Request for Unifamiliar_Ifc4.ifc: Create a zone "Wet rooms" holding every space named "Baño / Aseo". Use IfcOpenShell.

First a look at what the model holds.

```python
import ifcopenshell

model = ifcopenshell.open("Unifamiliar_Ifc4.ifc")
print(model.schema)
seen = {}
for space in model.by_type("IfcSpace"):
    seen[space.LongName] = seen.get(space.LongName, 0) + 1
for name, count in sorted(seen.items(), key=str):
    print(count, "x", name)
print("zones:", [z.Name for z in model.by_type("IfcZone")][:20])
```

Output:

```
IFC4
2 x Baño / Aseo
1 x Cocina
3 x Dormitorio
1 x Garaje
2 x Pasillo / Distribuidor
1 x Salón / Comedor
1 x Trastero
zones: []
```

```python
import ifcopenshell
import ifcopenshell.api.group
import ifcopenshell.api.root

model = ifcopenshell.open("Unifamiliar_Ifc4.ifc")

names = {"Baño / Aseo"}
spaces = [s for s in model.by_type("IfcSpace") if s.LongName in names]

zone = ifcopenshell.api.root.create_entity(model, ifc_class="IfcZone", name="Wet rooms")
ifcopenshell.api.group.assign_group(model, products=spaces, group=zone)
print(len(spaces), "spaces in", zone.Name)

model.write("Unifamiliar_Ifc4_updated.ifc")
```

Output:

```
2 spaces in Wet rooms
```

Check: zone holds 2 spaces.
